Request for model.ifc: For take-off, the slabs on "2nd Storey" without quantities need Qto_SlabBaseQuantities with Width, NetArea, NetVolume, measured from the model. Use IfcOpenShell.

First a look at what the model holds.

```python
import ifcopenshell
import ifcopenshell.util.element
import ifcopenshell.util.unit

model = ifcopenshell.open("model.ifc")
print(model.schema)
for unit_type in ("LENGTHUNIT", "AREAUNIT", "VOLUMEUNIT"):
    print(unit_type, ifcopenshell.util.unit.calculate_unit_scale(model, unit_type))
storey = next(s for s in model.by_type("IfcBuildingStorey") if s.Name == "2nd Storey")
slabs = [e for e in ifcopenshell.util.element.get_decomposition(storey) if e.is_a("IfcSlab")]
for e in sorted(slabs, key=lambda e: e.id()):
    print(e.id(), e.is_a(), e.Name, list(ifcopenshell.util.element.get_psets(e, qtos_only=True)), sep=" | ")
```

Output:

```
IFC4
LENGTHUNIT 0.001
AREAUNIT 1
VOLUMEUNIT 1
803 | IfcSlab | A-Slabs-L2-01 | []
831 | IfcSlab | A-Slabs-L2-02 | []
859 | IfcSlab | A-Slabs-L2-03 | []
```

```python
import ifcopenshell
import ifcopenshell.api.pset
import ifcopenshell.geom
import ifcopenshell.util.element
import ifcopenshell.util.shape
import ifcopenshell.util.unit

model = ifcopenshell.open("model.ifc")
unit_scale = ifcopenshell.util.unit.calculate_unit_scale(model)
area_scale = ifcopenshell.util.unit.calculate_unit_scale(model, "AREAUNIT")
volume_scale = ifcopenshell.util.unit.calculate_unit_scale(model, "VOLUMEUNIT")
settings = ifcopenshell.geom.settings()

storey = next(s for s in model.by_type("IfcBuildingStorey") if s.Name == "2nd Storey")
slabs = [e for e in ifcopenshell.util.element.get_decomposition(storey) if e.is_a("IfcSlab")]

for e in sorted(slabs, key=lambda e: e.id()):
    if ifcopenshell.util.element.get_psets(e, qtos_only=True, should_inherit=False):
        continue
    # Geometry comes back in metres, in the element's own axes.
    shape = ifcopenshell.geom.create_shape(settings, e)
    values = {
        "Width": ifcopenshell.util.shape.get_z(shape.geometry) / unit_scale,
        "NetArea": ifcopenshell.util.shape.get_footprint_area(shape.geometry) / area_scale,
        "NetVolume": ifcopenshell.util.shape.get_volume(shape.geometry) / volume_scale,
    }
    qto = ifcopenshell.api.pset.add_qto(model, product=e, name="Qto_SlabBaseQuantities")
    ifcopenshell.api.pset.edit_qto(model, qto=qto, properties=values)
    print(e.id(), {k: round(v, 3) for k, v in values.items()})

model.write("model_rev.ifc")
```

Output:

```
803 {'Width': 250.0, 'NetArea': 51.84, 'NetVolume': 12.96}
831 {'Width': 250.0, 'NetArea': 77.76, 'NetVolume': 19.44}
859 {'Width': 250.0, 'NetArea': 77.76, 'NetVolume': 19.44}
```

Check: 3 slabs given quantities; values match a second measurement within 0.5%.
